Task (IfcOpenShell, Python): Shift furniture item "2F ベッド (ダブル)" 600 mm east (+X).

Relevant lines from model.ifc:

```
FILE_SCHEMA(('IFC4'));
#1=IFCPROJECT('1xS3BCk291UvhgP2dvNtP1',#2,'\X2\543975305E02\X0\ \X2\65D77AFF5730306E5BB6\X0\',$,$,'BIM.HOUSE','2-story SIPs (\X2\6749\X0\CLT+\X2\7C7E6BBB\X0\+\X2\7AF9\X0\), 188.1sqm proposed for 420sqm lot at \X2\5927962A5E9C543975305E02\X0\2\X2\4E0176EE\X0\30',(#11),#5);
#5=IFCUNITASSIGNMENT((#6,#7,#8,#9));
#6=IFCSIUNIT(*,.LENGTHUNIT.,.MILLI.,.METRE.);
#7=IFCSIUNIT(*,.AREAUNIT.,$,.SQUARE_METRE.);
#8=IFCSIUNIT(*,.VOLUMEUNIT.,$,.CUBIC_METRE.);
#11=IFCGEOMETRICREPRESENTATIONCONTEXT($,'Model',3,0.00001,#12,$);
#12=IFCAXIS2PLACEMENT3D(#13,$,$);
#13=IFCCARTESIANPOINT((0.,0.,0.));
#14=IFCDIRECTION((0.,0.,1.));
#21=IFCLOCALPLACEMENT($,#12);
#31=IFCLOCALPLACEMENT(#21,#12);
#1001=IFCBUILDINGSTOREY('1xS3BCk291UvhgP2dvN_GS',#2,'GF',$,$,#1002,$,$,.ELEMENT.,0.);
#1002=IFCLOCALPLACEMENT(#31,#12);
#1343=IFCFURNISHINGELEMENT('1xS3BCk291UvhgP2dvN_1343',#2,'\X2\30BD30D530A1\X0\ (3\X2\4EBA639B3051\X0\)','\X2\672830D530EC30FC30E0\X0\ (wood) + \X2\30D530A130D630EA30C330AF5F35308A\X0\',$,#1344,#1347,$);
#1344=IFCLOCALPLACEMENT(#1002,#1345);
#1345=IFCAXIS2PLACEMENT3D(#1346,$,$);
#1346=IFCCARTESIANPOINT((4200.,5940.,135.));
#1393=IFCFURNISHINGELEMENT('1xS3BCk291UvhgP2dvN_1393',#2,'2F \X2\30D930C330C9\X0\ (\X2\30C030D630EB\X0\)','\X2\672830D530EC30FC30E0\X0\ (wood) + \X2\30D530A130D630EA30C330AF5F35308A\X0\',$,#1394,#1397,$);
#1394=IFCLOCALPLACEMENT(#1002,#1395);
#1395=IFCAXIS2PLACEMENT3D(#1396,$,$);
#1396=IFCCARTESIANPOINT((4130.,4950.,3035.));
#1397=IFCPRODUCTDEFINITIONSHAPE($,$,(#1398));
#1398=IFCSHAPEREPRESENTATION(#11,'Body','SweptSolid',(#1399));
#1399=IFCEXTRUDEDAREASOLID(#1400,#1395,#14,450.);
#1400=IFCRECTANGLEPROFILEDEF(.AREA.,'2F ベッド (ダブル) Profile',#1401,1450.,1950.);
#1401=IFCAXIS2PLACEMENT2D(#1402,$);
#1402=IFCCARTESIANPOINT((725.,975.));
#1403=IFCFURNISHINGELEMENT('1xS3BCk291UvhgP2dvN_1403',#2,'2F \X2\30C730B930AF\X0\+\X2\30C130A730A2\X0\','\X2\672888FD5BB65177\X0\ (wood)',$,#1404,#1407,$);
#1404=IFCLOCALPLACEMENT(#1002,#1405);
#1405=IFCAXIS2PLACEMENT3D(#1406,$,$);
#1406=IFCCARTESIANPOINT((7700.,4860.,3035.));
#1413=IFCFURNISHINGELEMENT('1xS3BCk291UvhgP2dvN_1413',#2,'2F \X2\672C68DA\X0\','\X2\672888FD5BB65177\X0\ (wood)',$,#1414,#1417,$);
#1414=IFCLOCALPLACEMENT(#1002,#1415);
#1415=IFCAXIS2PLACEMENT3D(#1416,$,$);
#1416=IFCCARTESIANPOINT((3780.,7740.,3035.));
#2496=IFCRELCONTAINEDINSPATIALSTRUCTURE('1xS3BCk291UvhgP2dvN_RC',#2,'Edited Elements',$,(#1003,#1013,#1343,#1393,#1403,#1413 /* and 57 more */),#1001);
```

```python
import ifcopenshell
import ifcopenshell.api.geometry
import ifcopenshell.util.placement
import ifcopenshell.util.unit

model = ifcopenshell.open("model.ifc")
unit_scale = ifcopenshell.util.unit.calculate_unit_scale(model)

item = model.by_id(1393)
matrix = ifcopenshell.util.placement.get_local_placement(item.ObjectPlacement)
matrix[0, 3] += 0.6 / unit_scale
ifcopenshell.api.geometry.edit_object_placement(model, product=item, matrix=matrix, is_si=False)

print(ifcopenshell.util.placement.get_local_placement(item.ObjectPlacement).round(3) + 0.0)

model.write("model-out.ifc")
```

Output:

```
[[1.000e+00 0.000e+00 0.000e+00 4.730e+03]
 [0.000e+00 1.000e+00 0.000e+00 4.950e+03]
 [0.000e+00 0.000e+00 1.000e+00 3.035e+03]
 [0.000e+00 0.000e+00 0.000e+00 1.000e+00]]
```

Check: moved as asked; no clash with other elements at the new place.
